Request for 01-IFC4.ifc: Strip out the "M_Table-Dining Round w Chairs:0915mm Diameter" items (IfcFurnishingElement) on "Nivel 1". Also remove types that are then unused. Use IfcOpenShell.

First a look at what the model holds.

```python
import ifcopenshell
import ifcopenshell.util.element

model = ifcopenshell.open("01-IFC4.ifc")
print(model.schema)
storey = next(s for s in model.by_type("IfcBuildingStorey") if s.Name == "Nivel 1")
furniture = [e for e in ifcopenshell.util.element.get_decomposition(storey) if e.is_a("IfcFurnishingElement")]
seen = {}
for e in furniture:
    element_type = ifcopenshell.util.element.get_type(e)
    name = element_type.Name if element_type not in (None, e) else None
    seen[name] = seen.get(name, 0) + 1
for name, count in sorted(seen.items(), key=str):
    print(count, "x", name)
```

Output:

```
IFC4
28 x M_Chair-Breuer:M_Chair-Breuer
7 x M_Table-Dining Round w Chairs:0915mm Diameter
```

```python
import ifcopenshell
import ifcopenshell.api.root
import ifcopenshell.util.element

model = ifcopenshell.open("01-IFC4.ifc")

storey = next(s for s in model.by_type("IfcBuildingStorey") if s.Name == "Nivel 1")
furniture = [e for e in ifcopenshell.util.element.get_decomposition(storey) if e.is_a("IfcFurnishingElement")]
targets = [e for e in furniture if (t := ifcopenshell.util.element.get_type(e)) not in (None, e) and t.Name == "M_Table-Dining Round w Chairs:0915mm Diameter"]
types = {ifcopenshell.util.element.get_type(e) for e in targets} - {None, *targets}

for e in targets:
    ifcopenshell.api.root.remove_product(model, product=e)
print(len(targets), "removed")

unused = [t for t in types if not ifcopenshell.util.element.get_types(t)]
for t in unused:
    ifcopenshell.api.root.remove_product(model, product=t)
print(len(unused), "unused types removed")

model.write("01-IFC4_updated.ifc")
```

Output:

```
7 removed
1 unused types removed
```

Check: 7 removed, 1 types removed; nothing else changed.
